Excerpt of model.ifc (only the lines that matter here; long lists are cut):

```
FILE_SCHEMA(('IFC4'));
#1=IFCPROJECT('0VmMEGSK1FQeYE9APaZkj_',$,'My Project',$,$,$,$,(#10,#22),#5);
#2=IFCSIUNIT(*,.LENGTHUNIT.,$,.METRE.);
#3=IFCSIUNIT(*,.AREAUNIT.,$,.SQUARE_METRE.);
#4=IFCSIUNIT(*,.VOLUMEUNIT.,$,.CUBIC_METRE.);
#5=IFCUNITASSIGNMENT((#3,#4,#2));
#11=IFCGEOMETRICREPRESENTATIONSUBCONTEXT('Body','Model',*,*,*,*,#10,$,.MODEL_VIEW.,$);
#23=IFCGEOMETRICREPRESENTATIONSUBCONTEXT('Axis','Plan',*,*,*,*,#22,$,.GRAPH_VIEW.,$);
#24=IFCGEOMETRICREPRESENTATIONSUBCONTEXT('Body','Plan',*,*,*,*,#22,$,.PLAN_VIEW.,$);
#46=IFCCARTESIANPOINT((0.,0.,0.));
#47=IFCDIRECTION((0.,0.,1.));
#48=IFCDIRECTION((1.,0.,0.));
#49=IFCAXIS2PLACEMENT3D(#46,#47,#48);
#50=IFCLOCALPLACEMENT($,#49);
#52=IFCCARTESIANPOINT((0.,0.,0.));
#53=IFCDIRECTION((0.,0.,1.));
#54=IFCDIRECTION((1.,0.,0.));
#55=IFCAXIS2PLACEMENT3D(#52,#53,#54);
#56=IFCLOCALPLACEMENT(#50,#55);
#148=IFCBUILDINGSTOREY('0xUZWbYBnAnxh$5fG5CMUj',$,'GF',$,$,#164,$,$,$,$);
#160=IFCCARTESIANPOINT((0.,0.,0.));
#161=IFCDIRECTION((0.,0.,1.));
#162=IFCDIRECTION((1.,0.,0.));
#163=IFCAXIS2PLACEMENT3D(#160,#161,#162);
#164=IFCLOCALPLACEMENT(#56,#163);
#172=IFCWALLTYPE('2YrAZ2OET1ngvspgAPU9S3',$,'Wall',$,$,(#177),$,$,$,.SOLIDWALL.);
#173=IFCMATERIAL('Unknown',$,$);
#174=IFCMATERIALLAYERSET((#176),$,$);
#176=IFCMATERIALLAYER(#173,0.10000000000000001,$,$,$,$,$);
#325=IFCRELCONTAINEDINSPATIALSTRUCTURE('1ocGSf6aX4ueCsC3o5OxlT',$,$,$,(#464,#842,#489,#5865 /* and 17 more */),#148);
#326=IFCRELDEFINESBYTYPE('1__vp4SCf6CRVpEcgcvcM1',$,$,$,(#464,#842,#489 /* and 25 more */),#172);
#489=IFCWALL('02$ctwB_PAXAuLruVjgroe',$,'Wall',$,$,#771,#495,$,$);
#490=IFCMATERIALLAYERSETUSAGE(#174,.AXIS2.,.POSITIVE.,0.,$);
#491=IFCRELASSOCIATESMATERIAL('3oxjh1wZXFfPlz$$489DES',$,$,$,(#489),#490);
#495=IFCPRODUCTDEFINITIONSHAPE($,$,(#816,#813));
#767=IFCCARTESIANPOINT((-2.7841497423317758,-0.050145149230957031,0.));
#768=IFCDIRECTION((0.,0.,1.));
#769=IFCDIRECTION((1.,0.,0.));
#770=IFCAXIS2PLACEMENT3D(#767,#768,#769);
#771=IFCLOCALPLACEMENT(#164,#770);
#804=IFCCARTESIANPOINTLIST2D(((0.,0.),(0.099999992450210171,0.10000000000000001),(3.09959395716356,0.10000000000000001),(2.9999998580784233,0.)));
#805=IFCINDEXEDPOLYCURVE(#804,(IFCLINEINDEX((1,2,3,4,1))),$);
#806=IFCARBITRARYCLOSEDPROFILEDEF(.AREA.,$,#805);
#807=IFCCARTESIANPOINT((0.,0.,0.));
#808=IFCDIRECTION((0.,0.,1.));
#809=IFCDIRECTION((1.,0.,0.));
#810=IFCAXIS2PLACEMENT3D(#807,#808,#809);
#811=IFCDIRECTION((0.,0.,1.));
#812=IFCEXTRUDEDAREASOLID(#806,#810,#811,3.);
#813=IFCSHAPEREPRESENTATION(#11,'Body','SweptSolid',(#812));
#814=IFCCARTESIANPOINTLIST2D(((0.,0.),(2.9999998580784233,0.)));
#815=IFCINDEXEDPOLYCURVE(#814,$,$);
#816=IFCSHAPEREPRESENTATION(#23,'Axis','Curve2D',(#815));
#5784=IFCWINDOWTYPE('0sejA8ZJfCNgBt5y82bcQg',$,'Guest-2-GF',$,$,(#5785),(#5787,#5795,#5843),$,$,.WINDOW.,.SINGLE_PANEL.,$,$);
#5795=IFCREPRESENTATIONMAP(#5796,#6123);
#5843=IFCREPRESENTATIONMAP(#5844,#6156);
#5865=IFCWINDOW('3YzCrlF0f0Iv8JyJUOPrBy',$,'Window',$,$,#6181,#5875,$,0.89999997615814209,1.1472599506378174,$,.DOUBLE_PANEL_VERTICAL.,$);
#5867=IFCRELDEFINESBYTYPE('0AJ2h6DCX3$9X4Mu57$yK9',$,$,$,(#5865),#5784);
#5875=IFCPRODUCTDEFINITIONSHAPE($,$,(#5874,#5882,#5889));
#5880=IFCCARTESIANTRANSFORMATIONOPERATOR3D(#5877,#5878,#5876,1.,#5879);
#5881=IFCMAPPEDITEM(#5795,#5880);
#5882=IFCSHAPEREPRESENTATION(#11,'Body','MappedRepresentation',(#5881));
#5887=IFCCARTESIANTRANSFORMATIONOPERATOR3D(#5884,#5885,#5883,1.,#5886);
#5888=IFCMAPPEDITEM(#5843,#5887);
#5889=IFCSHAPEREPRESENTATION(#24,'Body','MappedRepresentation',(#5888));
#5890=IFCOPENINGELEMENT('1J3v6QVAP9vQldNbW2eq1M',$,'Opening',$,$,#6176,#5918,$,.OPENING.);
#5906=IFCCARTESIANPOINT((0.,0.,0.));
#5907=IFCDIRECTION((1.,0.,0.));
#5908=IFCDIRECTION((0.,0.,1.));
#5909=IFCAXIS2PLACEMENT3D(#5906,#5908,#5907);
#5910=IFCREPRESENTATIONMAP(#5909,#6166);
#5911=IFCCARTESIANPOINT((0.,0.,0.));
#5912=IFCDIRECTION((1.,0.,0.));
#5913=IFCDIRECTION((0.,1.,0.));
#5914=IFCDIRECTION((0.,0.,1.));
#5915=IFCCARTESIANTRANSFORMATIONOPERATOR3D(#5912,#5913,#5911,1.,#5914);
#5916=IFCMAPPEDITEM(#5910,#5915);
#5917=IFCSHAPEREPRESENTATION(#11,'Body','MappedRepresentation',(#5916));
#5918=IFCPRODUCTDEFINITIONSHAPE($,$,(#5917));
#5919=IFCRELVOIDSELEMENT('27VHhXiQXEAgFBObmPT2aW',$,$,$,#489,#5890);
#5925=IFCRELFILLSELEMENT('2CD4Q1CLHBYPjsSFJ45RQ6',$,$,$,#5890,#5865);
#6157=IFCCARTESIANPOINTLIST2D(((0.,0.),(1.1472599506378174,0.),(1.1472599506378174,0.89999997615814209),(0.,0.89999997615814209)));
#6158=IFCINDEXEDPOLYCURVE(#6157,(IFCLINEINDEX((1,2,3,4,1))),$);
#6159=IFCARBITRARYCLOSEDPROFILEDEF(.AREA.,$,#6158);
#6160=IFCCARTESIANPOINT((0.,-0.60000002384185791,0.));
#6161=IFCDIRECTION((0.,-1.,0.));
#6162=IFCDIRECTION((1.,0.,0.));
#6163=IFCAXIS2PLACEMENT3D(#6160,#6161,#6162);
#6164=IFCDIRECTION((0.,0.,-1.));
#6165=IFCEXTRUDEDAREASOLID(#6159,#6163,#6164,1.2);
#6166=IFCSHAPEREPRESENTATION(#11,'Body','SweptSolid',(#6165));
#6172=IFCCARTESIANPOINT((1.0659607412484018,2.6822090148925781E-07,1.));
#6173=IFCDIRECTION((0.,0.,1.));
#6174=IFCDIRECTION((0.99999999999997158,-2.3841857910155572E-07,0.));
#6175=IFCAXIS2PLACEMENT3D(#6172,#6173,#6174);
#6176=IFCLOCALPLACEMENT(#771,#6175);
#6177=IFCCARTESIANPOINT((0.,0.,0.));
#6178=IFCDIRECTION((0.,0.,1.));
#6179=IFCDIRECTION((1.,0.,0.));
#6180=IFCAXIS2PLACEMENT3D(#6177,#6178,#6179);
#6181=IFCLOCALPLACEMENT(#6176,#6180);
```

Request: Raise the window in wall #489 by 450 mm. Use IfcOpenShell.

```python
import numpy as np
import ifcopenshell
import ifcopenshell.api.geometry
import ifcopenshell.util.placement
import ifcopenshell.util.unit

model = ifcopenshell.open("model.ifc")
unit_scale = ifcopenshell.util.unit.calculate_unit_scale(model)

window = model.by_guid("3YzCrlF0f0Iv8JyJUOPrBy")
opening = window.FillsVoids[0].RelatingOpeningElement
dz = 0.45

shift = np.array([0.0, 0.0, dz])
# The window is placed relative to its opening, so it follows when the opening moves.
matrix = ifcopenshell.util.placement.get_local_placement(opening.ObjectPlacement)
matrix[:3, 3] += shift
ifcopenshell.api.geometry.edit_object_placement(
    model, product=opening, matrix=matrix, is_si=False, should_transform_children=True
)

print(f"moved by {dz * unit_scale:+.3f} m")

model.write("model_v2.ifc")
```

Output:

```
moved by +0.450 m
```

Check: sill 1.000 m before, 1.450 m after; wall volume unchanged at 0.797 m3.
